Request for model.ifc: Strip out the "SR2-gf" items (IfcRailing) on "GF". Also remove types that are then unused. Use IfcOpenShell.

First a look at what the model holds.

```python
import ifcopenshell
import ifcopenshell.util.element

model = ifcopenshell.open("model.ifc")
print(model.schema)
storey = next(s for s in model.by_type("IfcBuildingStorey") if s.Name == "GF")
railings = [e for e in ifcopenshell.util.element.get_decomposition(storey) if e.is_a("IfcRailing")]
seen = {}
for e in railings:
    element_type = ifcopenshell.util.element.get_type(e)
    name = element_type.Name if element_type not in (None, e) else None
    seen[name] = seen.get(name, 0) + 1
for name, count in sorted(seen.items(), key=str):
    print(count, "x", name)
```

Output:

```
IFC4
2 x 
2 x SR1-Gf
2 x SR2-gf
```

```python
import ifcopenshell
import ifcopenshell.api.root
import ifcopenshell.util.element

model = ifcopenshell.open("model.ifc")

storey = next(s for s in model.by_type("IfcBuildingStorey") if s.Name == "GF")
railings = [e for e in ifcopenshell.util.element.get_decomposition(storey) if e.is_a("IfcRailing")]
targets = [e for e in railings if (t := ifcopenshell.util.element.get_type(e)) not in (None, e) and t.Name == "SR2-gf"]
types = {ifcopenshell.util.element.get_type(e) for e in targets} - {None, *targets}

for e in targets:
    ifcopenshell.api.root.remove_product(model, product=e)
print(len(targets), "removed")

unused = [t for t in types if not ifcopenshell.util.element.get_types(t)]
for t in unused:
    ifcopenshell.api.root.remove_product(model, product=t)
print(len(unused), "unused types removed")

model.write("model_rev.ifc")
```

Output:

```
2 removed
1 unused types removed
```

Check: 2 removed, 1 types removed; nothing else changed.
